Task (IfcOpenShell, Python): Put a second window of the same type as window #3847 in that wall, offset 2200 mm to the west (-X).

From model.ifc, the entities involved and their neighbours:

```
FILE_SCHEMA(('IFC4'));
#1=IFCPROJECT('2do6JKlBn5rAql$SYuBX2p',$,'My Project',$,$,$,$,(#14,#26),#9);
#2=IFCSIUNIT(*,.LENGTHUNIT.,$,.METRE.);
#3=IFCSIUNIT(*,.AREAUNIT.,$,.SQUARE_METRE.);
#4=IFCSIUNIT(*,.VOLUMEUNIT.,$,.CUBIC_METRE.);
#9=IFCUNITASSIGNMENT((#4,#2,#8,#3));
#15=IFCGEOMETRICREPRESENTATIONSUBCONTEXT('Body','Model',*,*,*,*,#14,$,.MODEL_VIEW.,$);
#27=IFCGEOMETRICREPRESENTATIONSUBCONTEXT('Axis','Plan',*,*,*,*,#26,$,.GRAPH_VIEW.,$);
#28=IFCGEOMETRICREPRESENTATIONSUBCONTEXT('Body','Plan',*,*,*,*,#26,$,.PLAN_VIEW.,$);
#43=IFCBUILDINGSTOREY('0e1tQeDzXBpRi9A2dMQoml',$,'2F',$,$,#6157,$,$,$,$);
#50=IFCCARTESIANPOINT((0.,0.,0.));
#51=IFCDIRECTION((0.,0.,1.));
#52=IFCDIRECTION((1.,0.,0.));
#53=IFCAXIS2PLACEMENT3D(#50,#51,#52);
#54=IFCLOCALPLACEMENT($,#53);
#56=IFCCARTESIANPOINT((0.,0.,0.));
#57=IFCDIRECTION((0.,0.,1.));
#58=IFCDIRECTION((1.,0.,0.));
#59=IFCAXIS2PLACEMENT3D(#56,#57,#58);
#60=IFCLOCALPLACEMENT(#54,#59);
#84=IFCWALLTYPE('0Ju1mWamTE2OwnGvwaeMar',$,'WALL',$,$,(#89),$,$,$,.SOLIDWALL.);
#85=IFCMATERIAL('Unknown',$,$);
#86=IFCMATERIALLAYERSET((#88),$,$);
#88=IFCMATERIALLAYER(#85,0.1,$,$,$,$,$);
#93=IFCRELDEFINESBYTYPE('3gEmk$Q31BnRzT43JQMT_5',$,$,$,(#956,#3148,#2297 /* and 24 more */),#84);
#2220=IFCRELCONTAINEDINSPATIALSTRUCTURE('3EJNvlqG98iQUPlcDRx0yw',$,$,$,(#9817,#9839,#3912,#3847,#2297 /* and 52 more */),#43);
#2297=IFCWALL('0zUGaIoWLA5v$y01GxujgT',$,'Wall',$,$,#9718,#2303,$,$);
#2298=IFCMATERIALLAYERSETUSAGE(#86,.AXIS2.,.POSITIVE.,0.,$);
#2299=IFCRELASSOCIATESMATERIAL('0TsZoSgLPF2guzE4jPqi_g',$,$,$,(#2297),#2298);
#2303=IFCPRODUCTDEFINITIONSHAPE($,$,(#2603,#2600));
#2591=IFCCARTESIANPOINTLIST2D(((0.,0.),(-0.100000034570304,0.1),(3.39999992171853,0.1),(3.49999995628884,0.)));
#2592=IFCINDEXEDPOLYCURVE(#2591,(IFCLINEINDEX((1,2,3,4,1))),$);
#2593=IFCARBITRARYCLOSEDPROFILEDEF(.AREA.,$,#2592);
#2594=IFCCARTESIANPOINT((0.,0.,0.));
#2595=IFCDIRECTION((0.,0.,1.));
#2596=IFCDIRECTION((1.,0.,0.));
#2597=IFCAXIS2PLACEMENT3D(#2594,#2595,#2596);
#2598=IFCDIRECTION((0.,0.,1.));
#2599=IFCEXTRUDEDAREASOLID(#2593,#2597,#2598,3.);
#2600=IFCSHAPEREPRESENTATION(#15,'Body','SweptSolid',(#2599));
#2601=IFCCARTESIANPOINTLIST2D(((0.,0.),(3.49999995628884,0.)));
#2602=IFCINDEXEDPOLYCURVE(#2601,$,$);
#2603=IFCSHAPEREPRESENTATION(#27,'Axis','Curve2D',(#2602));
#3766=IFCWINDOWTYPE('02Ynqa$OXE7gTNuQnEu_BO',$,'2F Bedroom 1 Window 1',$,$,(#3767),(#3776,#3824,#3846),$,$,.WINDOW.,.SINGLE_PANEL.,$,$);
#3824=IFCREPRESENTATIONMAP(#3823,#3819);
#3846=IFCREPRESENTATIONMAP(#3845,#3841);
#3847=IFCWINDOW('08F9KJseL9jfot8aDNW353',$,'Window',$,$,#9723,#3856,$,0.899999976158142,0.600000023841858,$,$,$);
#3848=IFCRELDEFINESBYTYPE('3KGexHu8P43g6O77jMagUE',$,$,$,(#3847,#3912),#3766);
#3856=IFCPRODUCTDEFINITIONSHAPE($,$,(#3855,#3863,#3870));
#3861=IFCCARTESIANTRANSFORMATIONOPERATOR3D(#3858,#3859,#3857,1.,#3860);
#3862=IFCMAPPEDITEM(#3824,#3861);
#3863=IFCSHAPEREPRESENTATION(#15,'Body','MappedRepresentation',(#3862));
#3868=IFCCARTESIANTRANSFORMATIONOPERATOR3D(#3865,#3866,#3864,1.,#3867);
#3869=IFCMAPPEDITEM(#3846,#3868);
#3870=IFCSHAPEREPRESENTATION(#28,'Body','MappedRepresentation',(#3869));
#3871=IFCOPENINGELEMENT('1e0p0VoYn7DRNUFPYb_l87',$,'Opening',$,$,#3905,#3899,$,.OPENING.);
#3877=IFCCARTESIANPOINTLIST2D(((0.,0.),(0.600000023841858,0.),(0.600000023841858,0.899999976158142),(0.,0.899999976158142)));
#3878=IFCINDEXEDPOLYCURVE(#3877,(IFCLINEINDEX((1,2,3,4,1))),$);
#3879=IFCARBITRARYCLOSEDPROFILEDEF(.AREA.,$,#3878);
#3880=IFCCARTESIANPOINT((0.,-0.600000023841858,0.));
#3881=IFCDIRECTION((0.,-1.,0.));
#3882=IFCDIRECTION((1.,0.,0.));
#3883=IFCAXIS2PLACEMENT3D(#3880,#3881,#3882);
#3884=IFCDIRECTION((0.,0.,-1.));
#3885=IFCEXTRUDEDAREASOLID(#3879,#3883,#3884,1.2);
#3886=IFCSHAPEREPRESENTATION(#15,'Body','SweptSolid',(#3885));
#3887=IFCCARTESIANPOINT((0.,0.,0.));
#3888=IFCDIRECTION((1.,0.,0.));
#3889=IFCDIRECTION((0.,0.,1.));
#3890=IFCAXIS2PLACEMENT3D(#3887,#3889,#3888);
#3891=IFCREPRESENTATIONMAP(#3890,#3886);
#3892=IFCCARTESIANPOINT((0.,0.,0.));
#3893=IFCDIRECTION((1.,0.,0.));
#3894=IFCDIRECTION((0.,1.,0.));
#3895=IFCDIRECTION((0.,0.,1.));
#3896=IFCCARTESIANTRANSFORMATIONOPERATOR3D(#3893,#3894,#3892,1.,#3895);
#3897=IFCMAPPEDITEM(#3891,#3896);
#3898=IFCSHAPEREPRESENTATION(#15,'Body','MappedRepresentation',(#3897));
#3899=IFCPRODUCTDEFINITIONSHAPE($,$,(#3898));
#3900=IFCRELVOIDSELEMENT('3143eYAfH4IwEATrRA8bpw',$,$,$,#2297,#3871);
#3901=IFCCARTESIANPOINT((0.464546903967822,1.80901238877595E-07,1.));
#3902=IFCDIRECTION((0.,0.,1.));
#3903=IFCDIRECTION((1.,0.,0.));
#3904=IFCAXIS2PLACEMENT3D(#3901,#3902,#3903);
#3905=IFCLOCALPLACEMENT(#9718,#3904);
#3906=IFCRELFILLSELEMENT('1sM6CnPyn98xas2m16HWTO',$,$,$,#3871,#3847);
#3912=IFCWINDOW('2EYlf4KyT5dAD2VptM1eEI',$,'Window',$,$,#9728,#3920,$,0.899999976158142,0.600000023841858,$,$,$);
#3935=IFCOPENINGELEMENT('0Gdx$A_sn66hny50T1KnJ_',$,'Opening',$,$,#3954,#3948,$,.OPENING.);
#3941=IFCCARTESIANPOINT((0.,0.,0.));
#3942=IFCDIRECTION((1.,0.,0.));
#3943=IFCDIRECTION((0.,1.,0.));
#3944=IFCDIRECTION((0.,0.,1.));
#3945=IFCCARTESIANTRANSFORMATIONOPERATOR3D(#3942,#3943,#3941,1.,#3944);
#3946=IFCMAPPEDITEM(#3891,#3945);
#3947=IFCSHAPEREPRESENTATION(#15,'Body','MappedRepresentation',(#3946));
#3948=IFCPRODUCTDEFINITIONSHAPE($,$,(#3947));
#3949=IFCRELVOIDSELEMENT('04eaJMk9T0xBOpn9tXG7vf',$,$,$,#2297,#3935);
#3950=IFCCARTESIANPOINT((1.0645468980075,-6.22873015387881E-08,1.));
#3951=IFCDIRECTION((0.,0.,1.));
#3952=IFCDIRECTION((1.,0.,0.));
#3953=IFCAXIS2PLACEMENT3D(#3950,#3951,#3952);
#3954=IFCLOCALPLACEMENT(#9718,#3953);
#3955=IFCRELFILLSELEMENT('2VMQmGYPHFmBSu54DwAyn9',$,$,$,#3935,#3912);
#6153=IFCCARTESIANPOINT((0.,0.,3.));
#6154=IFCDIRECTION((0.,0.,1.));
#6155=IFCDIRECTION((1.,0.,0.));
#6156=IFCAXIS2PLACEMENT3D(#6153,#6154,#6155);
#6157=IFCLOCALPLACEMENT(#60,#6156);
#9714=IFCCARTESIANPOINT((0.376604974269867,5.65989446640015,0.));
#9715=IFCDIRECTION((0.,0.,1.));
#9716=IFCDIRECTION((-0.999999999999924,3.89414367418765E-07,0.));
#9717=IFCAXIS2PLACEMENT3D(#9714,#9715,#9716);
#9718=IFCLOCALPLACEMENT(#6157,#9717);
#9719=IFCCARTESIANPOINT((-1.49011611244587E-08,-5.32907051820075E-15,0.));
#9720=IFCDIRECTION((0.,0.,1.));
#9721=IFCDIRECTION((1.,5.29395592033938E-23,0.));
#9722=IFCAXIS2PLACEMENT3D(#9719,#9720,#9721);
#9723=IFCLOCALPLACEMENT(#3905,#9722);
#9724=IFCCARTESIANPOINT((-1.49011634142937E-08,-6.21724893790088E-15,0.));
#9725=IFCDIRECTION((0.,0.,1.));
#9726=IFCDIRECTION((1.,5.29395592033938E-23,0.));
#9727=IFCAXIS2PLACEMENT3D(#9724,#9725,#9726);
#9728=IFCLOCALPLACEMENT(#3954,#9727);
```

```python
import ifcopenshell
import ifcopenshell.api.feature
import ifcopenshell.api.geometry
import ifcopenshell.api.root
import ifcopenshell.geom
import ifcopenshell.util.element
import ifcopenshell.util.placement
import ifcopenshell.util.shape
import ifcopenshell.util.unit

model = ifcopenshell.open("model.ifc")
unit_scale = ifcopenshell.util.unit.calculate_unit_scale(model)
settings = ifcopenshell.geom.settings()


def volume(element):
    """Net volume in cubic metres, openings subtracted."""
    shape = ifcopenshell.geom.create_shape(settings, element)
    return ifcopenshell.util.shape.get_volume(shape.geometry)


window = model.by_guid("08F9KJseL9jfot8aDNW353")
opening = window.FillsVoids[0].RelatingOpeningElement
wall = opening.VoidsElements[0].RelatingBuildingElement
before = volume(wall)
shift = ifcopenshell.util.placement.get_local_placement(wall.ObjectPlacement)[:3, 0] * 2.2 / unit_scale

# copy_class copies the void relationship, type, container and properties, but no geometry.
new_opening = ifcopenshell.api.root.copy_class(model, product=opening)
new_opening.Representation = ifcopenshell.util.element.copy_deep(
    model, opening.Representation, exclude=["IfcGeometricRepresentationContext", "IfcRepresentationMap"]
)
new_window = ifcopenshell.api.root.copy_class(model, product=window)
new_window.Representation = ifcopenshell.util.element.copy_deep(
    model, window.Representation, exclude=["IfcGeometricRepresentationContext", "IfcRepresentationMap"]
)
ifcopenshell.api.feature.add_filling(model, opening=new_opening, element=new_window)

for old, new in ((opening, new_opening), (window, new_window)):
    matrix = ifcopenshell.util.placement.get_local_placement(old.ObjectPlacement)
    matrix[:3, 3] += shift
    ifcopenshell.api.geometry.edit_object_placement(model, product=new, matrix=matrix, is_si=False)

after = volume(wall)

print(f"wall volume {before:.3f} -> {after:.3f} m3")

model.write("model_rev.ifc")
```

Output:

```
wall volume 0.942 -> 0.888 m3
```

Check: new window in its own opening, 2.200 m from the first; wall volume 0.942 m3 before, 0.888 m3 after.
